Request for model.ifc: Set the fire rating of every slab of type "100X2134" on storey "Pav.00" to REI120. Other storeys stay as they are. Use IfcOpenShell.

First a look at what the model holds.

```python
import ifcopenshell
import ifcopenshell.util.element

model = ifcopenshell.open("model.ifc")
print(model.schema)
storey = next(s for s in model.by_type("IfcBuildingStorey") if s.Name == "Pav.00")
slabs = [e for e in ifcopenshell.util.element.get_decomposition(storey) if e.is_a("IfcSlab")]
seen = {}
for e in slabs:
    element_type = ifcopenshell.util.element.get_type(e)
    key = (element_type.Name if element_type != e and element_type else None, ifcopenshell.util.element.get_pset(e, "Pset_SlabCommon", "FireRating"))
    seen[key] = seen.get(key, 0) + 1
for (name, value), count in sorted(seen.items(), key=str):
    print(count, "x", name, "|", value)
```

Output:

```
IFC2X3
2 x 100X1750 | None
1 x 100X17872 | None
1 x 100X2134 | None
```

```python
import ifcopenshell
import ifcopenshell.api.pset
import ifcopenshell.util.element

model = ifcopenshell.open("model.ifc")

storey = next(s for s in model.by_type("IfcBuildingStorey") if s.Name == "Pav.00")
slabs = [e for e in ifcopenshell.util.element.get_decomposition(storey) if e.is_a("IfcSlab")]

count = 0
for e in slabs:
    element_type = ifcopenshell.util.element.get_type(e)
    if element_type in (None, e) or element_type.Name != "100X2134":
        continue
    found = ifcopenshell.util.element.get_pset(e, "Pset_SlabCommon", should_inherit=False)
    if found:
        pset = model.by_id(found["id"])
        if len(ifcopenshell.util.element.get_elements_by_pset(pset)) > 1:
            pset = ifcopenshell.api.pset.unshare_pset(model, products=[e], pset=pset)[0]
    else:
        pset = ifcopenshell.api.pset.add_pset(model, product=e, name="Pset_SlabCommon")
    ifcopenshell.api.pset.edit_pset(model, pset=pset, properties={"FireRating": "REI120"})
    count += 1

print(count, "slabs updated")

model.write("model_rev.ifc")
```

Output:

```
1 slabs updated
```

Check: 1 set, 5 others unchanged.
